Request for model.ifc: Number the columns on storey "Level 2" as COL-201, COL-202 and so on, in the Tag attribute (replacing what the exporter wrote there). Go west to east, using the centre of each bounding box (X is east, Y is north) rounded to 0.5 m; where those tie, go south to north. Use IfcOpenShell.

First a look at what the model holds.

```python
import ifcopenshell
import ifcopenshell.util.element
import ifcopenshell.util.placement

model = ifcopenshell.open("model.ifc")
print(model.schema)
storey = next(s for s in model.by_type("IfcBuildingStorey") if s.Name == "Level 2")
columns = [e for e in ifcopenshell.util.element.get_decomposition(storey) if e.is_a("IfcColumn")]
for e in sorted(columns, key=lambda e: e.id()):
    origin = ifcopenshell.util.placement.get_local_placement(e.ObjectPlacement)[:3, 3]
    print(e.id(), e.Tag, e.Name, origin.round(2) + 0.0, sep=" | ")
```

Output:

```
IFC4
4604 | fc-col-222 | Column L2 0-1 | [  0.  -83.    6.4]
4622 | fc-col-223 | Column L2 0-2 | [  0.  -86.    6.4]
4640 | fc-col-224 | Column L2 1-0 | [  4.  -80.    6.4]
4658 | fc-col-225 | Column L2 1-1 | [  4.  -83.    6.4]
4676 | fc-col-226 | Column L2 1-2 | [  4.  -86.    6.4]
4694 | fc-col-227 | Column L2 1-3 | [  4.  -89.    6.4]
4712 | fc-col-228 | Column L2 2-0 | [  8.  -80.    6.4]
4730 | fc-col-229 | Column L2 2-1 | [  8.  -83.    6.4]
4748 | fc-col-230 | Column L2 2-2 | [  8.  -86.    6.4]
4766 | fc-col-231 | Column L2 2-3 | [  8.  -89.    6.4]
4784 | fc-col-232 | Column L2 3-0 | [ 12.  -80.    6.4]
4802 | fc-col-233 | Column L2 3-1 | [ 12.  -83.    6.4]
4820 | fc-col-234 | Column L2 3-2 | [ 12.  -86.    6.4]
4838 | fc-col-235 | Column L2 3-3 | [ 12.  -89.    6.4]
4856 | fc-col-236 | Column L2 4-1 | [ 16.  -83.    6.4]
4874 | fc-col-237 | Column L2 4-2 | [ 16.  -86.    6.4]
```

```python
import ifcopenshell
import ifcopenshell.geom
import ifcopenshell.util.element
import ifcopenshell.util.shape

model = ifcopenshell.open("model.ifc")
settings = ifcopenshell.geom.settings()
settings.set("use-world-coords", True)


def centre(element):
    shape = ifcopenshell.geom.create_shape(settings, element)
    return ifcopenshell.util.shape.get_bbox_centroid(shape.geometry)


storey = next(s for s in model.by_type("IfcBuildingStorey") if s.Name == "Level 2")
columns = [e for e in ifcopenshell.util.element.get_decomposition(storey) if e.is_a("IfcColumn")]

# Insertion points can sit at a corner or the storey origin, so sort by the geometry (in metres).
centres = {e: centre(e) for e in columns}
columns.sort(key=lambda e: (round(centres[e][0] / 0.5), centres[e][1]))

for i, e in enumerate(columns, start=1):
    number = f"COL-2{i:02d}"
    e.Tag = number
    print(e.id(), number)

model.write("model_edited.ifc")
```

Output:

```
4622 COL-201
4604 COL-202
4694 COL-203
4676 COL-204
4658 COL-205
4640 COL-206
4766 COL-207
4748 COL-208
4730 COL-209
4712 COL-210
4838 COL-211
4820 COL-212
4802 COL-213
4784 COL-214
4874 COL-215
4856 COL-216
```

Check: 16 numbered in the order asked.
